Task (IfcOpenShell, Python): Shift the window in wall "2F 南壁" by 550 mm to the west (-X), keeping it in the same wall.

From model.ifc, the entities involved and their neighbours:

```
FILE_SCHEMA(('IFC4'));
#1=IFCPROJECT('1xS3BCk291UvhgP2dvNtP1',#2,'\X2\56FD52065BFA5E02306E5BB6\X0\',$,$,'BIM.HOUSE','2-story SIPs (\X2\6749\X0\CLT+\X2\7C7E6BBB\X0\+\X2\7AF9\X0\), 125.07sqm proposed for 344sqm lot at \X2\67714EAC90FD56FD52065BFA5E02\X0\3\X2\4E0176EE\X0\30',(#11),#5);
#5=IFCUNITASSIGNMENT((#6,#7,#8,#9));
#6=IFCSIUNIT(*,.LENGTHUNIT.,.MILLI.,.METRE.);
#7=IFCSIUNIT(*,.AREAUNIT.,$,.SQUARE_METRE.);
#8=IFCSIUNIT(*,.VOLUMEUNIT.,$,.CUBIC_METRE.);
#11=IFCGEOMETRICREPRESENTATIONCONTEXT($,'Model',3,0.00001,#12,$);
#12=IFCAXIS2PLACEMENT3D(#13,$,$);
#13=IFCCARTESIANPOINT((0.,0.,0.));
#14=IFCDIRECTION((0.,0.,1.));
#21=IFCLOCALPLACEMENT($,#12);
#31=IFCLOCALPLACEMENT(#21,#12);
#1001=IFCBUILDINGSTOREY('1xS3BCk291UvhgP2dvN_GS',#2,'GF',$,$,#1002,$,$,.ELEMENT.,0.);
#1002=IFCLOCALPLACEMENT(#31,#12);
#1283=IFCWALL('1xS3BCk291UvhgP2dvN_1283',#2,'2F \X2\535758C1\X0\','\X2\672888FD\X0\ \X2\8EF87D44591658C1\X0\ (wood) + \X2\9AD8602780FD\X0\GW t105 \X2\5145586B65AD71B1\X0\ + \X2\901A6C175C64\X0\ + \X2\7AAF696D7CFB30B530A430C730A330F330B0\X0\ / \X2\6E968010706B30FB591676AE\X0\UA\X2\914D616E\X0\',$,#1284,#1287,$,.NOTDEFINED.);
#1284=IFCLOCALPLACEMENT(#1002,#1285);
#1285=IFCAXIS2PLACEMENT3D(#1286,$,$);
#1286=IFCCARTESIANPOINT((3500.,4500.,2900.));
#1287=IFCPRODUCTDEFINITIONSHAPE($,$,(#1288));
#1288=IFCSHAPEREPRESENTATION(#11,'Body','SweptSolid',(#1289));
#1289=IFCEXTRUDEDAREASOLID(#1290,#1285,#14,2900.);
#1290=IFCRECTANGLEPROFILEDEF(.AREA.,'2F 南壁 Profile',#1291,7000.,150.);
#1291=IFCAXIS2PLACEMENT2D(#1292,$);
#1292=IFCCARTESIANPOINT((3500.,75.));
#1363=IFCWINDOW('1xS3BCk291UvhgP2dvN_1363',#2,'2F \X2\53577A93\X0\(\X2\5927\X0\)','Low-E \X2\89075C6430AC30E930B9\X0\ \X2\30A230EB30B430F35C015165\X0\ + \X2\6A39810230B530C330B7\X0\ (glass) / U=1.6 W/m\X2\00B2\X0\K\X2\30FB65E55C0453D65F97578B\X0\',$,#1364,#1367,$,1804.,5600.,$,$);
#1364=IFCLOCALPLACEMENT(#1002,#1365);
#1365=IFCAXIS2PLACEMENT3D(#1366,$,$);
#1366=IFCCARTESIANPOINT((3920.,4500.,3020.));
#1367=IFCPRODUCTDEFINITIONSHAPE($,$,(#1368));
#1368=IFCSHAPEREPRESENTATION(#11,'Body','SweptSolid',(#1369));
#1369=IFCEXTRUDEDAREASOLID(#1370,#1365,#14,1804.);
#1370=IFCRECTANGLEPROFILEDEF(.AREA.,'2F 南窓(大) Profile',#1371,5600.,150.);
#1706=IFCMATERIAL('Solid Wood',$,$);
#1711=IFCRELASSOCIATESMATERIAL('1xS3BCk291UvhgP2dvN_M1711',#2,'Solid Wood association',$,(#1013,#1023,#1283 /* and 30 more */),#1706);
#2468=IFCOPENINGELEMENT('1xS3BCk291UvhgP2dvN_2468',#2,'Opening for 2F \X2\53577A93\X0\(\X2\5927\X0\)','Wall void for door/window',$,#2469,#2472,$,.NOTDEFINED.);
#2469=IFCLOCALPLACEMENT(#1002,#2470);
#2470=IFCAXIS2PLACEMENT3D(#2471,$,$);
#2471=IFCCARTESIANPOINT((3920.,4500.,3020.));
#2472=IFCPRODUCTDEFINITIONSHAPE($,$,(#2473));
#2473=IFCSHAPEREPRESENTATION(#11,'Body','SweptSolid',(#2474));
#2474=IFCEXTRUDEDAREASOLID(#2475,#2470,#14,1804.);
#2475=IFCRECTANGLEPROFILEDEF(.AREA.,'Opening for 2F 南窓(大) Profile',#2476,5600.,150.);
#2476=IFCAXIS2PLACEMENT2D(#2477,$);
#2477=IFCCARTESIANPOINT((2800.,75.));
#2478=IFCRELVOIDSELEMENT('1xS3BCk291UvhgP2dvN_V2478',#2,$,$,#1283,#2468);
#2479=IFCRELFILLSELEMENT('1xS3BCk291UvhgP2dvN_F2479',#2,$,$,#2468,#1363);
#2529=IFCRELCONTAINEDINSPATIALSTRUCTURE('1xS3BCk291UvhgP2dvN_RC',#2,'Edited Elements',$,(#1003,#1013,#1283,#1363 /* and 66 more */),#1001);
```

```python
import ifcopenshell
import ifcopenshell.api.geometry
import ifcopenshell.util.placement

model = ifcopenshell.open("model.ifc")

window = model.by_guid("1xS3BCk291UvhgP2dvN_1363")
opening = window.FillsVoids[0].RelatingOpeningElement
wall = opening.VoidsElements[0].RelatingBuildingElement

wall_matrix = ifcopenshell.util.placement.get_local_placement(wall.ObjectPlacement)
shift = wall_matrix[:3, 0] * -550.0
before = ifcopenshell.util.placement.get_local_placement(window.ObjectPlacement)[:3, 3].copy()

# The window is not placed relative to its opening, so move both.
for product in (opening, window):
    matrix = ifcopenshell.util.placement.get_local_placement(product.ObjectPlacement)
    matrix[:3, 3] += shift
    ifcopenshell.api.geometry.edit_object_placement(model, product=product, matrix=matrix, is_si=False)

after = ifcopenshell.util.placement.get_local_placement(window.ObjectPlacement)[:3, 3]
print("window moved by", (after - before).round(3) + 0.0)

model.write("model_rev.ifc")
```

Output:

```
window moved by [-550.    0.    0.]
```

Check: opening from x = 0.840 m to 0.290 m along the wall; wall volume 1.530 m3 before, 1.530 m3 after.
